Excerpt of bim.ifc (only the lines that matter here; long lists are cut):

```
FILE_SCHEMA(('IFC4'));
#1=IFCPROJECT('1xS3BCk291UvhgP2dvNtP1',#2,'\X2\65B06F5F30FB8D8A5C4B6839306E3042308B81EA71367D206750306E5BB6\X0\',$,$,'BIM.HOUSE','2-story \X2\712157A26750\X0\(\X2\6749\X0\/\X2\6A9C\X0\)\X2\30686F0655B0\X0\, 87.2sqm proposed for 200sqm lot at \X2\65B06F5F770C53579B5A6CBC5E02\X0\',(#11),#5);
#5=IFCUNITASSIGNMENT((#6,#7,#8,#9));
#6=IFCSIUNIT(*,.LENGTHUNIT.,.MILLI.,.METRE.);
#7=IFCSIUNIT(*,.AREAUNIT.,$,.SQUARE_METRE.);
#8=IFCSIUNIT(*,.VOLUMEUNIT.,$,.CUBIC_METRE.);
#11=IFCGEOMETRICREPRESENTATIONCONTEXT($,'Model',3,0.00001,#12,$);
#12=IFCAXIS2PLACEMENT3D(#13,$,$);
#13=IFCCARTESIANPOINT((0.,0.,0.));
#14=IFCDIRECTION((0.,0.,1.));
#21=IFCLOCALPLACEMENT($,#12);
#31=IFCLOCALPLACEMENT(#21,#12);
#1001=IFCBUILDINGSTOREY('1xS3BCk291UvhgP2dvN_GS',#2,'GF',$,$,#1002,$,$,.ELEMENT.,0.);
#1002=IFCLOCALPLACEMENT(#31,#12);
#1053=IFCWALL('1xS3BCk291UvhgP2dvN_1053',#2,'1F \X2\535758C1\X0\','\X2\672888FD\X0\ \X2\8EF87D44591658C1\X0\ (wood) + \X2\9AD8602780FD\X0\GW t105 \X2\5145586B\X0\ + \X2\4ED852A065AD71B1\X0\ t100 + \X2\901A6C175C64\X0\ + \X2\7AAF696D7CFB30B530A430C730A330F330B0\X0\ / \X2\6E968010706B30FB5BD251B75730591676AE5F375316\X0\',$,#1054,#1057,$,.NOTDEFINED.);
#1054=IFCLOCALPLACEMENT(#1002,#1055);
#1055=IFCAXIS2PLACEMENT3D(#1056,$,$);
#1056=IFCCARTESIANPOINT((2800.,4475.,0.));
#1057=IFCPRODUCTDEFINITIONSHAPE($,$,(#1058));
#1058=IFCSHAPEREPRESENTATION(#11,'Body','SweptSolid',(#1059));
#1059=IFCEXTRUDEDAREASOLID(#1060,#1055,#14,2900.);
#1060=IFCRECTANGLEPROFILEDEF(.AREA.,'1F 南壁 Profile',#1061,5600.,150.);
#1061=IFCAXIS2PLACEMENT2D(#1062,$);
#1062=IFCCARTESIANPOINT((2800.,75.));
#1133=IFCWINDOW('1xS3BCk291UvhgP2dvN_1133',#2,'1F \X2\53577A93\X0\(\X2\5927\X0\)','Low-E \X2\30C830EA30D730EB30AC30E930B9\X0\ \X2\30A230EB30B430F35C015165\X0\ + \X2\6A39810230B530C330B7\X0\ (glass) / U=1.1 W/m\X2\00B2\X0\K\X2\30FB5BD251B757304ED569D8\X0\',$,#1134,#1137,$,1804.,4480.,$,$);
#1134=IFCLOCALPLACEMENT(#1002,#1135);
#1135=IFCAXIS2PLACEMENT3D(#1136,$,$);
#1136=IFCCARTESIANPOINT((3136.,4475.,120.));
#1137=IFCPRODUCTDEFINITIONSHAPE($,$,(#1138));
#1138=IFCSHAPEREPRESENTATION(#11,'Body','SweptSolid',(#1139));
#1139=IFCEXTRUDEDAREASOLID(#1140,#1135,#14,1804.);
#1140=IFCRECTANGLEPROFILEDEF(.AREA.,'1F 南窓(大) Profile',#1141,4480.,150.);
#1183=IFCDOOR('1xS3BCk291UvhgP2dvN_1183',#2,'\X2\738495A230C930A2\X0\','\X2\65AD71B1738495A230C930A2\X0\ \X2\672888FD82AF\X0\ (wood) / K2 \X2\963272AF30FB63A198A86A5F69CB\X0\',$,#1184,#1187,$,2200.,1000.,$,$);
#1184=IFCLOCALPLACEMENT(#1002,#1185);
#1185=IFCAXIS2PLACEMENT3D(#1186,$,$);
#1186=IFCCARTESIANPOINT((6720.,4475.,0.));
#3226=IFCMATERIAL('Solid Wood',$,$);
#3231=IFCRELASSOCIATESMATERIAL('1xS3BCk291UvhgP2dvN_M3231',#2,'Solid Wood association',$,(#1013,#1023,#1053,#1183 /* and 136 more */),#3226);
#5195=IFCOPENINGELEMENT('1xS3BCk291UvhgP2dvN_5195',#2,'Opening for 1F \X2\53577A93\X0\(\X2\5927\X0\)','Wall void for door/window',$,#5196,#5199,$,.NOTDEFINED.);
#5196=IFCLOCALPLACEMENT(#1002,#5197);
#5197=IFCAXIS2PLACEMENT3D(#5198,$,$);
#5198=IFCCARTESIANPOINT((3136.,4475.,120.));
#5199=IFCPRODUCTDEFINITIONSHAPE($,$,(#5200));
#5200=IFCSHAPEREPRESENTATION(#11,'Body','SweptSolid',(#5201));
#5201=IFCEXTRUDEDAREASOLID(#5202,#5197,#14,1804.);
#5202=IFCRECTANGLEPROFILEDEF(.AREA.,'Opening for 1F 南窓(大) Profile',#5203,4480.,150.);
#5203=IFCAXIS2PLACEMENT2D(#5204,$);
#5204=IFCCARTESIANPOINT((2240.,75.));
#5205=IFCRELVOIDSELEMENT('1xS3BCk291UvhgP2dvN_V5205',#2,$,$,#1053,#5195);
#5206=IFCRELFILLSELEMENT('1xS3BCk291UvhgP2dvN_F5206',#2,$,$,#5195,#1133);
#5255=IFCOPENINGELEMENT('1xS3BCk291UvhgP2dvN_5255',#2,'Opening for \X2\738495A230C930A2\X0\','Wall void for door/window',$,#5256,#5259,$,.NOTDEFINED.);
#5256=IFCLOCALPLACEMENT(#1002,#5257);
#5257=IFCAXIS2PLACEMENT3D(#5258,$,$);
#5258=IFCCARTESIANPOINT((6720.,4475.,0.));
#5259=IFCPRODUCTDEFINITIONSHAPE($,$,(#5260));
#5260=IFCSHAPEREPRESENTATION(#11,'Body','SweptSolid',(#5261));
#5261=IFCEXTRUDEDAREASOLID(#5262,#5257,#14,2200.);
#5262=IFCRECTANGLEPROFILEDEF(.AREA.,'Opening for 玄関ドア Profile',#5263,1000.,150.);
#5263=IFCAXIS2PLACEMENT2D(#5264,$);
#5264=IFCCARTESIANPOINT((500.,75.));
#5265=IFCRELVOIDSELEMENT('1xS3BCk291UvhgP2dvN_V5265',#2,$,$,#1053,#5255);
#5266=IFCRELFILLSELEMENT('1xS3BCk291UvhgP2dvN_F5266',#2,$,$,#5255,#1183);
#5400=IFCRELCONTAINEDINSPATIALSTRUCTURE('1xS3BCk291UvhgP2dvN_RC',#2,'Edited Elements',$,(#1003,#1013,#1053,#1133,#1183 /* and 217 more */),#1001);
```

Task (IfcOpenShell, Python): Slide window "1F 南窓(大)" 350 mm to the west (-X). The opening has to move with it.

```python
import ifcopenshell
import ifcopenshell.api.geometry
import ifcopenshell.util.placement
import ifcopenshell.util.unit

model = ifcopenshell.open("bim.ifc")
unit_scale = ifcopenshell.util.unit.calculate_unit_scale(model)

window = model.by_id(1133)
opening = window.FillsVoids[0].RelatingOpeningElement
wall = opening.VoidsElements[0].RelatingBuildingElement

wall_matrix = ifcopenshell.util.placement.get_local_placement(wall.ObjectPlacement)
shift = wall_matrix[:3, 0] * -0.35 / unit_scale
before = ifcopenshell.util.placement.get_local_placement(window.ObjectPlacement)[:3, 3].copy()

# The window is not placed relative to its opening, so move both.
for product in (opening, window):
    matrix = ifcopenshell.util.placement.get_local_placement(product.ObjectPlacement)
    matrix[:3, 3] += shift
    ifcopenshell.api.geometry.edit_object_placement(model, product=product, matrix=matrix, is_si=False)

after = ifcopenshell.util.placement.get_local_placement(window.ObjectPlacement)[:3, 3]
print("window moved by", (after - before).round(3) + 0.0)

model.write("bim_updated.ifc")
```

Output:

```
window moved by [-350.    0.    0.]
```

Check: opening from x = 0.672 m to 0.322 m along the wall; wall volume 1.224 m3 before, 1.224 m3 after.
